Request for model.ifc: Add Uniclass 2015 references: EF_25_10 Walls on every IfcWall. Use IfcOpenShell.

First a look at what the model holds.

```python
import ifcopenshell

model = ifcopenshell.open("model.ifc")
print(model.schema)
print("classifications:", [c.Name for c in model.by_type("IfcClassification")])
for ifc_class in ("IfcDoor", "IfcRoof", "IfcStair", "IfcWall", "IfcWindow"):
    print(ifc_class, len(model.by_type(ifc_class)))
```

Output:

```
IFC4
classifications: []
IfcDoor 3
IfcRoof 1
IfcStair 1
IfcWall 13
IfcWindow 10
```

```python
import ifcopenshell
import ifcopenshell.api.classification

model = ifcopenshell.open("model.ifc")

system = ifcopenshell.api.classification.add_classification(model, classification="Uniclass 2015")

codes = {
    "IfcWall": ("EF_25_10", "Walls"),
}
for ifc_class, (code, name) in codes.items():
    products = model.by_type(ifc_class)
    ifcopenshell.api.classification.add_reference(
        model, products=products, classification=system, identification=code, name=name
    )
    print(code, len(products))

model.write("model_edited.ifc")
```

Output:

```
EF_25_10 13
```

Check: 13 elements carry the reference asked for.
